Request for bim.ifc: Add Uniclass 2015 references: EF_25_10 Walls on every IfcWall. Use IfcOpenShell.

First a look at what the model holds.

```python
import ifcopenshell

model = ifcopenshell.open("bim.ifc")
print(model.schema)
print("classifications:", [c.Name for c in model.by_type("IfcClassification")])
for ifc_class in ("IfcDoor", "IfcRoof", "IfcStair", "IfcWall", "IfcWindow"):
    print(ifc_class, len(model.by_type(ifc_class)))
```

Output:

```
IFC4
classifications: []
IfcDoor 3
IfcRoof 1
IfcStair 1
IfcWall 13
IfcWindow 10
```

```python
import ifcopenshell
import ifcopenshell.api.classification

model = ifcopenshell.open("bim.ifc")

system = ifcopenshell.api.classification.add_classification(model, classification="Uniclass 2015")

codes = {
    "IfcWall": ("EF_25_10", "Walls"),
}
for ifc_class, (code, name) in codes.items():
    products = model.by_type(ifc_class)
    ifcopenshell.api.classification.add_reference(
        model, products=products, classification=system, identification=code, name=name
    )
    print(code, len(products))

model.write("bim_rev.ifc")
```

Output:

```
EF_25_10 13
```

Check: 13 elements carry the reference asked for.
